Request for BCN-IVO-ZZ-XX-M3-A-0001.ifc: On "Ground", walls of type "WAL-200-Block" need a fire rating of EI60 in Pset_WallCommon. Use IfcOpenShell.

First a look at what the model holds.

```python
import ifcopenshell
import ifcopenshell.util.element

model = ifcopenshell.open("BCN-IVO-ZZ-XX-M3-A-0001.ifc")
print(model.schema)
storey = next(s for s in model.by_type("IfcBuildingStorey") if s.Name == "Ground")
walls = [e for e in ifcopenshell.util.element.get_decomposition(storey) if e.is_a("IfcWall")]
seen = {}
for e in walls:
    element_type = ifcopenshell.util.element.get_type(e)
    key = (element_type.Name if element_type != e and element_type else None, ifcopenshell.util.element.get_pset(e, "Pset_WallCommon", "FireRating"))
    seen[key] = seen.get(key, 0) + 1
for (name, value), count in sorted(seen.items(), key=str):
    print(count, "x", name, "|", value)
```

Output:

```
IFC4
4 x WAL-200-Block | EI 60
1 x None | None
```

```python
import ifcopenshell
import ifcopenshell.api.pset
import ifcopenshell.util.element

model = ifcopenshell.open("BCN-IVO-ZZ-XX-M3-A-0001.ifc")

storey = next(s for s in model.by_type("IfcBuildingStorey") if s.Name == "Ground")
walls = [e for e in ifcopenshell.util.element.get_decomposition(storey) if e.is_a("IfcWall")]

count = 0
for e in walls:
    element_type = ifcopenshell.util.element.get_type(e)
    if element_type in (None, e) or element_type.Name != "WAL-200-Block":
        continue
    # add_pset returns the element's existing set when there is one.
    pset = ifcopenshell.api.pset.add_pset(model, product=e, name="Pset_WallCommon")
    ifcopenshell.api.pset.edit_pset(model, pset=pset, properties={"FireRating": "EI60"})
    count += 1

print(count, "walls updated")

model.write("BCN-IVO-ZZ-XX-M3-A-0001_updated.ifc")
```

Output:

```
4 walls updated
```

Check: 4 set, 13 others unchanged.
